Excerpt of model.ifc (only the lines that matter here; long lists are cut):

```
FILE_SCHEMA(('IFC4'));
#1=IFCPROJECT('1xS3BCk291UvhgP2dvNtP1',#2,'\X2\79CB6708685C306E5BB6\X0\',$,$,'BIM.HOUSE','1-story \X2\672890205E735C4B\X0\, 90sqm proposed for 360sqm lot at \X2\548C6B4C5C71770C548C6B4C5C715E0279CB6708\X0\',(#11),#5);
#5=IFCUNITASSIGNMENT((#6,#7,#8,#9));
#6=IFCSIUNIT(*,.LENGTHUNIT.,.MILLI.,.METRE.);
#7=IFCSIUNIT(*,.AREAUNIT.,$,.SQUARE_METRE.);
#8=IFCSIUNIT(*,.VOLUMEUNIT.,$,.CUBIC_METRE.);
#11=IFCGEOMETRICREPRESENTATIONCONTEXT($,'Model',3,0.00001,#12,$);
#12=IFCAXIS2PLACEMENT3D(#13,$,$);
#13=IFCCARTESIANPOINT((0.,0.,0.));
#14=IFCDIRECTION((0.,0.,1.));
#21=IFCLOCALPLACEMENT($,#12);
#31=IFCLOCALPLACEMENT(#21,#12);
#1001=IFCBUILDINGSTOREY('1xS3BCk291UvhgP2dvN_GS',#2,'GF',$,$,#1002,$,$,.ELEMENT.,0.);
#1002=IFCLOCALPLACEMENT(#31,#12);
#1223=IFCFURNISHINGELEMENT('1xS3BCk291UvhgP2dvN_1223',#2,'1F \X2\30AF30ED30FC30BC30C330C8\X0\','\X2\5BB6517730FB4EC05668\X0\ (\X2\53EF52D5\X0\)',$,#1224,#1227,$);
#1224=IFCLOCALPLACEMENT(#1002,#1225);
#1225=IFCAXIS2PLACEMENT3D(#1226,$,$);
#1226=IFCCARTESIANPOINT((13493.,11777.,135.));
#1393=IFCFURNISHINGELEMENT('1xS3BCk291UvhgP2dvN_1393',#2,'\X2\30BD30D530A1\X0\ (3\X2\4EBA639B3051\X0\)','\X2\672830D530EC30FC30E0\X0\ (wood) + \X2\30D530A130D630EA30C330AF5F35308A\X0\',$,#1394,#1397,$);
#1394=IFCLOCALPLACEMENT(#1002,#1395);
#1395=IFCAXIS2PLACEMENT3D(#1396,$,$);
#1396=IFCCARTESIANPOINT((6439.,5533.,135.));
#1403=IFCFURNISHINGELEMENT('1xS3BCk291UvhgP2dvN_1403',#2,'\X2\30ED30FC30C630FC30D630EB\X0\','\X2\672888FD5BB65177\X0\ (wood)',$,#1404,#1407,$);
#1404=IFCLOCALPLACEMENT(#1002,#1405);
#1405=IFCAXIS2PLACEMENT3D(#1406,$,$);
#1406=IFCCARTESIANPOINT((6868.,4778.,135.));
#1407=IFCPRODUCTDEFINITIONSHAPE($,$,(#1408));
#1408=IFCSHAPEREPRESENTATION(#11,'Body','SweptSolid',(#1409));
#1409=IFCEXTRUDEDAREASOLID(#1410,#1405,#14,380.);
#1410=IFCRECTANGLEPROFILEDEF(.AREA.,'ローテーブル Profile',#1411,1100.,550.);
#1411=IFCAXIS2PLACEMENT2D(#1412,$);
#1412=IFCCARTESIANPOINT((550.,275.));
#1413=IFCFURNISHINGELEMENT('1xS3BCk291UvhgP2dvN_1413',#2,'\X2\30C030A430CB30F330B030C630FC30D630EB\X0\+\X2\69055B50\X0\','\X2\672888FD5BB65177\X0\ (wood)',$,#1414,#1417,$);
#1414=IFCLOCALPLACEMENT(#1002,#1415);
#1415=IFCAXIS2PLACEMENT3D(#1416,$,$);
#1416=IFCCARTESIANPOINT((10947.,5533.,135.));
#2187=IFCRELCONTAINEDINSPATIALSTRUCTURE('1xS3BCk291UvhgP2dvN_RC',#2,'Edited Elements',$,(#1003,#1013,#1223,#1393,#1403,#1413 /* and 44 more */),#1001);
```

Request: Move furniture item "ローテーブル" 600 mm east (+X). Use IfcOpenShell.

```python
import ifcopenshell
import ifcopenshell.api.geometry
import ifcopenshell.util.placement

model = ifcopenshell.open("model.ifc")

item = model.by_guid("1xS3BCk291UvhgP2dvN_1403")
matrix = ifcopenshell.util.placement.get_local_placement(item.ObjectPlacement)
matrix[0, 3] += 600.0
ifcopenshell.api.geometry.edit_object_placement(model, product=item, matrix=matrix, is_si=False)

print(ifcopenshell.util.placement.get_local_placement(item.ObjectPlacement).round(3) + 0.0)

model.write("model-out.ifc")
```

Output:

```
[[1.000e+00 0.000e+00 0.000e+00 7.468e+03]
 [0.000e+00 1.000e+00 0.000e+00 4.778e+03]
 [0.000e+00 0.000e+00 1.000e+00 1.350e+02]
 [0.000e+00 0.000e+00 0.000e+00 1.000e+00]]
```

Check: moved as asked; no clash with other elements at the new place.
